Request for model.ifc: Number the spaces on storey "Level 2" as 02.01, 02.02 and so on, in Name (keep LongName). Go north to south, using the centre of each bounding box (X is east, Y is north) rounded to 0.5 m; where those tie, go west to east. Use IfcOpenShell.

First a look at what the model holds.

```python
import ifcopenshell
import ifcopenshell.util.element
import ifcopenshell.util.placement

model = ifcopenshell.open("model.ifc")
print(model.schema)
storey = next(s for s in model.by_type("IfcBuildingStorey") if s.Name == "Level 2")
spaces = [e for e in ifcopenshell.util.element.get_decomposition(storey) if e.is_a("IfcSpace")]
for e in sorted(spaces, key=lambda e: e.id()):
    origin = ifcopenshell.util.placement.get_local_placement(e.ObjectPlacement)[:3, 3]
    print(e.id(), e.Name, e.LongName, origin.round(2) + 0.0, sep=" | ")
```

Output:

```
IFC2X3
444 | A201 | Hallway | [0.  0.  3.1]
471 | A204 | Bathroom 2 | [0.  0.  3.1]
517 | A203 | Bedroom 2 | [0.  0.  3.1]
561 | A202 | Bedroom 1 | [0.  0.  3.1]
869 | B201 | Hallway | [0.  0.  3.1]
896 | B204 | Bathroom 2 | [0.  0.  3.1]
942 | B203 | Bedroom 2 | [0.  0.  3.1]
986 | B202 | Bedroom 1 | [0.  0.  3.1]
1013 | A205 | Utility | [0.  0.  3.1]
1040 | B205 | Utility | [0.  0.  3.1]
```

```python
import ifcopenshell
import ifcopenshell.geom
import ifcopenshell.util.element
import ifcopenshell.util.shape

model = ifcopenshell.open("model.ifc")
settings = ifcopenshell.geom.settings()
settings.set("use-world-coords", True)


def centre(element):
    shape = ifcopenshell.geom.create_shape(settings, element)
    return ifcopenshell.util.shape.get_bbox_centroid(shape.geometry)


storey = next(s for s in model.by_type("IfcBuildingStorey") if s.Name == "Level 2")
spaces = [e for e in ifcopenshell.util.element.get_decomposition(storey) if e.is_a("IfcSpace")]

# Insertion points can sit at a corner or the storey origin, so sort by the geometry (in metres).
centres = {e: centre(e) for e in spaces}
spaces.sort(key=lambda e: (-round(centres[e][1] / 0.5), centres[e][0]))

for i, e in enumerate(spaces, start=1):
    number = f"02.{i:02d}"
    e.Name = number
    print(e.id(), number)

model.write("model_edited.ifc")
```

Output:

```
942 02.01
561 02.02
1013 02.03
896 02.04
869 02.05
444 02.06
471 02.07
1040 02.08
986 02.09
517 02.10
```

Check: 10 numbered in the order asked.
